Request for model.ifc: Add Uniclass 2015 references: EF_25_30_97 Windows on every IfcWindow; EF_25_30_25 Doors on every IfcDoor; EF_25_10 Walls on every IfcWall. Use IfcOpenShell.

First a look at what the model holds.

```python
import ifcopenshell

model = ifcopenshell.open("model.ifc")
print(model.schema)
print("classifications:", [c.Name for c in model.by_type("IfcClassification")])
for ifc_class in ("IfcDoor", "IfcRoof", "IfcStair", "IfcWall", "IfcWindow"):
    print(ifc_class, len(model.by_type(ifc_class)))
```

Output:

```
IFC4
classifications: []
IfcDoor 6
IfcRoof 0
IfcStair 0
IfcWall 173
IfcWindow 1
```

```python
import ifcopenshell
import ifcopenshell.api.classification

model = ifcopenshell.open("model.ifc")

system = ifcopenshell.api.classification.add_classification(model, classification="Uniclass 2015")

codes = {
    "IfcWindow": ("EF_25_30_97", "Windows"),
    "IfcDoor": ("EF_25_30_25", "Doors"),
    "IfcWall": ("EF_25_10", "Walls"),
}
for ifc_class, (code, name) in codes.items():
    products = model.by_type(ifc_class)
    ifcopenshell.api.classification.add_reference(
        model, products=products, classification=system, identification=code, name=name
    )
    print(code, len(products))

model.write("model_rev.ifc")
```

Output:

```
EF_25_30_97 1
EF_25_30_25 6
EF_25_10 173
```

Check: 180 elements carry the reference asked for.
